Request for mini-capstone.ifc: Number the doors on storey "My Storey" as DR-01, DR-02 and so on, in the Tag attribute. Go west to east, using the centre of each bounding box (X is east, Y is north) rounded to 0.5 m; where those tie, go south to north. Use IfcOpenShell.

First a look at what the model holds.

```python
import ifcopenshell
import ifcopenshell.util.element
import ifcopenshell.util.placement

model = ifcopenshell.open("mini-capstone.ifc")
print(model.schema)
storey = next(s for s in model.by_type("IfcBuildingStorey") if s.Name == "My Storey")
doors = [e for e in ifcopenshell.util.element.get_decomposition(storey) if e.is_a("IfcDoor")]
for e in sorted(doors, key=lambda e: e.id()):
    origin = ifcopenshell.util.placement.get_local_placement(e.ObjectPlacement)[:3, 3]
    print(e.id(), e.Tag, e.Name, origin.round(2) + 0.0, sep=" | ")
```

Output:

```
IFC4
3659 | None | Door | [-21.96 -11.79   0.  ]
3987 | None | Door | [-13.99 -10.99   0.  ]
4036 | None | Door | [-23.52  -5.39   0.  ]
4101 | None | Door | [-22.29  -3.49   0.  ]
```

```python
import ifcopenshell
import ifcopenshell.geom
import ifcopenshell.util.element
import ifcopenshell.util.shape

model = ifcopenshell.open("mini-capstone.ifc")
settings = ifcopenshell.geom.settings()
settings.set("use-world-coords", True)


def centre(element):
    shape = ifcopenshell.geom.create_shape(settings, element)
    return ifcopenshell.util.shape.get_bbox_centroid(shape.geometry)


storey = next(s for s in model.by_type("IfcBuildingStorey") if s.Name == "My Storey")
doors = [e for e in ifcopenshell.util.element.get_decomposition(storey) if e.is_a("IfcDoor")]

# Insertion points can sit at a corner or the storey origin, so sort by the geometry (in metres).
centres = {e: centre(e) for e in doors}
doors.sort(key=lambda e: (round(centres[e][0] / 0.5), centres[e][1]))

for i, e in enumerate(doors, start=1):
    number = f"DR-{i:02d}"
    e.Tag = number
    print(e.id(), number)

model.write("mini-capstone_rev.ifc")
```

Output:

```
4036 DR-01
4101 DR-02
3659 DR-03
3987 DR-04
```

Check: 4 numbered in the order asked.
